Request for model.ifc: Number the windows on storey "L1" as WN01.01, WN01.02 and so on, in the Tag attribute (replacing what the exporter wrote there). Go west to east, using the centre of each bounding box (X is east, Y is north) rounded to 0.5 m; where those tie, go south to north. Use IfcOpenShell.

First a look at what the model holds.

```python
import ifcopenshell
import ifcopenshell.util.element
import ifcopenshell.util.placement

model = ifcopenshell.open("model.ifc")
print(model.schema)
storey = next(s for s in model.by_type("IfcBuildingStorey") if s.Name == "L1")
windows = [e for e in ifcopenshell.util.element.get_decomposition(storey) if e.is_a("IfcWindow")]
for e in sorted(windows, key=lambda e: e.id()):
    origin = ifcopenshell.util.placement.get_local_placement(e.ObjectPlacement)[:3, 3]
    print(e.id(), e.Tag, e.Name, origin.round(2) + 0.0, sep=" | ")
```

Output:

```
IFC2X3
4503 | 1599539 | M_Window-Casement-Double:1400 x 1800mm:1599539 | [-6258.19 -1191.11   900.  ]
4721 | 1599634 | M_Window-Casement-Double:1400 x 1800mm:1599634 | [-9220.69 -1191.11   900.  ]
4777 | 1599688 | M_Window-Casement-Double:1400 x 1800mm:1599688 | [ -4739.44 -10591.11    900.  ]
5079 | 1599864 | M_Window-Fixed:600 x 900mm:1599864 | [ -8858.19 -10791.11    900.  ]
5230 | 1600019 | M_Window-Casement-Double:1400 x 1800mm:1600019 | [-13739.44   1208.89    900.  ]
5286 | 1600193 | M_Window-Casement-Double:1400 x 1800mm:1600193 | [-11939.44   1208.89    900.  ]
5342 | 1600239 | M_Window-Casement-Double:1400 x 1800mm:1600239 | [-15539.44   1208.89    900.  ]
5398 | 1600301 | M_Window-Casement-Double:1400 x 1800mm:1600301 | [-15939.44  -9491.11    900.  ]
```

```python
import ifcopenshell
import ifcopenshell.geom
import ifcopenshell.util.element
import ifcopenshell.util.shape

model = ifcopenshell.open("model.ifc")
settings = ifcopenshell.geom.settings()
settings.set("use-world-coords", True)


def centre(element):
    shape = ifcopenshell.geom.create_shape(settings, element)
    return ifcopenshell.util.shape.get_bbox_centroid(shape.geometry)


storey = next(s for s in model.by_type("IfcBuildingStorey") if s.Name == "L1")
windows = [e for e in ifcopenshell.util.element.get_decomposition(storey) if e.is_a("IfcWindow")]

# Insertion points can sit at a corner or the storey origin, so sort by the geometry (in metres).
centres = {e: centre(e) for e in windows}
windows.sort(key=lambda e: (round(centres[e][0] / 0.5), centres[e][1]))

for i, e in enumerate(windows, start=1):
    number = f"WN01.{i:02d}"
    e.Tag = number
    print(e.id(), number)

model.write("model_updated.ifc")
```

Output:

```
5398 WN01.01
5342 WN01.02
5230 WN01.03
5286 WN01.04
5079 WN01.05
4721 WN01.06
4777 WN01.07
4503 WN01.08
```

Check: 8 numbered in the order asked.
